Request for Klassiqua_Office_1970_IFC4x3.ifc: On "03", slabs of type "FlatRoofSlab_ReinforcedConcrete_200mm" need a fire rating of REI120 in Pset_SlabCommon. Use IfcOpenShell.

First a look at what the model holds.

```python
import ifcopenshell
import ifcopenshell.util.element

model = ifcopenshell.open("Klassiqua_Office_1970_IFC4x3.ifc")
print(model.schema)
storey = next(s for s in model.by_type("IfcBuildingStorey") if s.Name == "03")
slabs = [e for e in ifcopenshell.util.element.get_decomposition(storey) if e.is_a("IfcSlab")]
seen = {}
for e in slabs:
    element_type = ifcopenshell.util.element.get_type(e)
    key = (element_type.Name if element_type != e and element_type else None, ifcopenshell.util.element.get_pset(e, "Pset_SlabCommon", "FireRating"))
    seen[key] = seen.get(key, 0) + 1
for (name, value), count in sorted(seen.items(), key=str):
    print(count, "x", name, "|", value)
```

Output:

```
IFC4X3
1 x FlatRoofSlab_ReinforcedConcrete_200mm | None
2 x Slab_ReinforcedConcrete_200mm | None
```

```python
import ifcopenshell
import ifcopenshell.api.pset
import ifcopenshell.util.element

model = ifcopenshell.open("Klassiqua_Office_1970_IFC4x3.ifc")

storey = next(s for s in model.by_type("IfcBuildingStorey") if s.Name == "03")
slabs = [e for e in ifcopenshell.util.element.get_decomposition(storey) if e.is_a("IfcSlab")]

count = 0
for e in slabs:
    element_type = ifcopenshell.util.element.get_type(e)
    if element_type in (None, e) or element_type.Name != "FlatRoofSlab_ReinforcedConcrete_200mm":
        continue
    # add_pset returns the element's existing set when there is one.
    pset = ifcopenshell.api.pset.add_pset(model, product=e, name="Pset_SlabCommon")
    ifcopenshell.api.pset.edit_pset(model, pset=pset, properties={"FireRating": "REI120"})
    count += 1

print(count, "slabs updated")

model.write("Klassiqua_Office_1970_IFC4x3_rev.ifc")
```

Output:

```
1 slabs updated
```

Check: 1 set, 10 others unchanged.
